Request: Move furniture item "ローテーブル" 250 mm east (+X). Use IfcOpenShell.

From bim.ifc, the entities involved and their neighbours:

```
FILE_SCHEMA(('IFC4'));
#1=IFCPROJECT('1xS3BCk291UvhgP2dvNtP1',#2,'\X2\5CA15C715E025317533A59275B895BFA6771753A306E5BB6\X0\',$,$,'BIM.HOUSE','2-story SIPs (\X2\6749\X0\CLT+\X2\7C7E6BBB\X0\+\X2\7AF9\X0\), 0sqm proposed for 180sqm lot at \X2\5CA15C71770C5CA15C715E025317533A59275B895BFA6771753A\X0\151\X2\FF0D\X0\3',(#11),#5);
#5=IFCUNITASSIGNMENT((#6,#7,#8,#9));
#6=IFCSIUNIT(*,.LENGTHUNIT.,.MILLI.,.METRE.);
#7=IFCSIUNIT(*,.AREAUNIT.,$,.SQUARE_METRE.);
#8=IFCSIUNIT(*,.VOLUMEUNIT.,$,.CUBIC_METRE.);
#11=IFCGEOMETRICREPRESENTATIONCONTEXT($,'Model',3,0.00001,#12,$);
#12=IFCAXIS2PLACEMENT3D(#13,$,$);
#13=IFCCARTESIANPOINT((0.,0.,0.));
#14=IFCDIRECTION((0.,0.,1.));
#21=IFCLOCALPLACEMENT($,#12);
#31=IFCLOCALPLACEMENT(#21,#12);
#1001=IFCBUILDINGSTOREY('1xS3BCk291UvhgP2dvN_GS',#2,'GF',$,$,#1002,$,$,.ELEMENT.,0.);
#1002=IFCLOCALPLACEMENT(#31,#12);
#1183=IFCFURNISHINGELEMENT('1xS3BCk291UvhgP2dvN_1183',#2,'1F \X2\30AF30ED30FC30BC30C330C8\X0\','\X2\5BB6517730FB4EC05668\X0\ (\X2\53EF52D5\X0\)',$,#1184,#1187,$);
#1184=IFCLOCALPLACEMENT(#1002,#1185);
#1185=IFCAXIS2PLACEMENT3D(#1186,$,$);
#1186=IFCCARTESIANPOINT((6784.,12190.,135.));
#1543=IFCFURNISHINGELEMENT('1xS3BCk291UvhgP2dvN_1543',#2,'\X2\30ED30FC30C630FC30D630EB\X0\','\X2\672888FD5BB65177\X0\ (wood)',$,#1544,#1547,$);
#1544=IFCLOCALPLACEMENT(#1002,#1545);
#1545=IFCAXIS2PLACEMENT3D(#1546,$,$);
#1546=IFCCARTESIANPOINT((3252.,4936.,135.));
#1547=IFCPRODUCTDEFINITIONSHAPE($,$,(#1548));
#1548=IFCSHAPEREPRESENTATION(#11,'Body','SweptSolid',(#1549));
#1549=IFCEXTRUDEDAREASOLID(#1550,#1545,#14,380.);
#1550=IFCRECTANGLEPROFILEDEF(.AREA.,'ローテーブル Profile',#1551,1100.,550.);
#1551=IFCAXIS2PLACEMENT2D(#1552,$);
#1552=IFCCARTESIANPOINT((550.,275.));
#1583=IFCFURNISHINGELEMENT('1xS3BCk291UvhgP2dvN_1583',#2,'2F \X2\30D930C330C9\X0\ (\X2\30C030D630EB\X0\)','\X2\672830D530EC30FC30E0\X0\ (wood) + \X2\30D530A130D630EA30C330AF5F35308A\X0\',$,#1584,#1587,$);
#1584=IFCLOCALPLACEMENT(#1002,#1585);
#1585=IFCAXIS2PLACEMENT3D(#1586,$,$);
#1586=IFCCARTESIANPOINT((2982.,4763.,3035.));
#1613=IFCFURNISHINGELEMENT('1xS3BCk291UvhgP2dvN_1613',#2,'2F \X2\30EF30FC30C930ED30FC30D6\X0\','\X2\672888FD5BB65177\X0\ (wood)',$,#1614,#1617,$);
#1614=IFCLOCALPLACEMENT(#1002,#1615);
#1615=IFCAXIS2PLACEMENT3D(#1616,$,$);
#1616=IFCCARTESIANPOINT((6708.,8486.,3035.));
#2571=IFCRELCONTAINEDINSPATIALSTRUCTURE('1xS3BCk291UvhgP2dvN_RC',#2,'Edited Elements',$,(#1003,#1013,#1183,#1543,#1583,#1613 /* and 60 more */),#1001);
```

```python
import ifcopenshell
import ifcopenshell.api.geometry
import ifcopenshell.util.placement
import ifcopenshell.util.unit

model = ifcopenshell.open("bim.ifc")
unit_scale = ifcopenshell.util.unit.calculate_unit_scale(model)

item = model.by_guid("1xS3BCk291UvhgP2dvN_1543")
matrix = ifcopenshell.util.placement.get_local_placement(item.ObjectPlacement)
matrix[0, 3] += 0.25 / unit_scale
ifcopenshell.api.geometry.edit_object_placement(model, product=item, matrix=matrix, is_si=False)

print(ifcopenshell.util.placement.get_local_placement(item.ObjectPlacement).round(3) + 0.0)

model.write("bim_rev.ifc")
```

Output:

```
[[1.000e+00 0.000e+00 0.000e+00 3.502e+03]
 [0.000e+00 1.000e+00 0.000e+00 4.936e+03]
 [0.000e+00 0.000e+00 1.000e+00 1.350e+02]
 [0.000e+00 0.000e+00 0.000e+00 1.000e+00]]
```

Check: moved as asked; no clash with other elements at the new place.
